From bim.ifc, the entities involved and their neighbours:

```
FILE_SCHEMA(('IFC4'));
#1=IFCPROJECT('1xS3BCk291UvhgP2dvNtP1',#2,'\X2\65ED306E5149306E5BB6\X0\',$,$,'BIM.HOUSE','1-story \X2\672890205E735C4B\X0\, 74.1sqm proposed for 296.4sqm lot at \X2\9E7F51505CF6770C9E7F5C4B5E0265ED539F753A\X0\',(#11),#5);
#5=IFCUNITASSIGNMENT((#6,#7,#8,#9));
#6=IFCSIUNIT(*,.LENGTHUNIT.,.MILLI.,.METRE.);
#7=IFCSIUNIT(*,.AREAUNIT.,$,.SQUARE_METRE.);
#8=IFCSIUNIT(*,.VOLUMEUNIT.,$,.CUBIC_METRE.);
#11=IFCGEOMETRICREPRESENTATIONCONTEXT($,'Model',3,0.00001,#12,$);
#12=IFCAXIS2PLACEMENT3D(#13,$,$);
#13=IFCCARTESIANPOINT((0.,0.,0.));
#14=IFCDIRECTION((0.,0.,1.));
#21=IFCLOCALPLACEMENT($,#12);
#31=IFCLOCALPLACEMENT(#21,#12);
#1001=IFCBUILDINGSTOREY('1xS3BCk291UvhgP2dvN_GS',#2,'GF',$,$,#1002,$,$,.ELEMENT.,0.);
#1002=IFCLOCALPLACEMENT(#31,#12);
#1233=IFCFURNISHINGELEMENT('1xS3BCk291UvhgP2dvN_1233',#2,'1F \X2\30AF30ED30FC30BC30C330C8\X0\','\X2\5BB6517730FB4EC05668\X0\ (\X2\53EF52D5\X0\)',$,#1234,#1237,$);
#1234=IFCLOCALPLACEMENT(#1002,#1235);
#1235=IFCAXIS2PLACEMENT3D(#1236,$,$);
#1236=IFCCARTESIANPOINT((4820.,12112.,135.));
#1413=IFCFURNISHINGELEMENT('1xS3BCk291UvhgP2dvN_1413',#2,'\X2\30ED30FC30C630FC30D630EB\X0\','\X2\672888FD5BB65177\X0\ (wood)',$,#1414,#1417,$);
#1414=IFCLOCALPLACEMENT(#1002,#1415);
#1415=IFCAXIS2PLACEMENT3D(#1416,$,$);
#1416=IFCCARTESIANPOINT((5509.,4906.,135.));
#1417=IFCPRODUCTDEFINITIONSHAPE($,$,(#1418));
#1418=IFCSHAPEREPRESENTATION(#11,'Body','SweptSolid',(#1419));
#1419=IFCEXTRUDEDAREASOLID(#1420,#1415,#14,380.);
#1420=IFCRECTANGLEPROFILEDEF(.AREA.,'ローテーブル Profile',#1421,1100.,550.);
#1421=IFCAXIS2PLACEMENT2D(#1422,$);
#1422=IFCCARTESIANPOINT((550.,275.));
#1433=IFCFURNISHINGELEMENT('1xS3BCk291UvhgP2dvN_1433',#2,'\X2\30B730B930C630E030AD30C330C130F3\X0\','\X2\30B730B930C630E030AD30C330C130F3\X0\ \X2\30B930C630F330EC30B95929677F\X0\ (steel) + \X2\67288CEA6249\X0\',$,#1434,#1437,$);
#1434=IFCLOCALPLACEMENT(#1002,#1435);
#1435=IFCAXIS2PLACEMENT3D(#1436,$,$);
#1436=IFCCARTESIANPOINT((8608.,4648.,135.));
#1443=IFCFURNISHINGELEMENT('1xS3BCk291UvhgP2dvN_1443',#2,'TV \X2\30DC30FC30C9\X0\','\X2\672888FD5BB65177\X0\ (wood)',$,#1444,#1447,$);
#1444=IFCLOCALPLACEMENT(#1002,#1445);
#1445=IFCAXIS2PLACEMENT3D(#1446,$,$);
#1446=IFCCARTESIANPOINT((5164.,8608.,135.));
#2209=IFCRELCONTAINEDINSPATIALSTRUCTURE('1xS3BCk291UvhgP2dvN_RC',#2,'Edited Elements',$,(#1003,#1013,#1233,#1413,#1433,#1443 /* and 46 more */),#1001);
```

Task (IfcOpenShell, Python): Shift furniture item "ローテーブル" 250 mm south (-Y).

```python
import ifcopenshell
import ifcopenshell.api.geometry
import ifcopenshell.util.placement

model = ifcopenshell.open("bim.ifc")

item = model.by_guid("1xS3BCk291UvhgP2dvN_1413")
matrix = ifcopenshell.util.placement.get_local_placement(item.ObjectPlacement)
matrix[1, 3] -= 250.0
ifcopenshell.api.geometry.edit_object_placement(model, product=item, matrix=matrix, is_si=False)

print(ifcopenshell.util.placement.get_local_placement(item.ObjectPlacement).round(3) + 0.0)

model.write("bim_edited.ifc")
```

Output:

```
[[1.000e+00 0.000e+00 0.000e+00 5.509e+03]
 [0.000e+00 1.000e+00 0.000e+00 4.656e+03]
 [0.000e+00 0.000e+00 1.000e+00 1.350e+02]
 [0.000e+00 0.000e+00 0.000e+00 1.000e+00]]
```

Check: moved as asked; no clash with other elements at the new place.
